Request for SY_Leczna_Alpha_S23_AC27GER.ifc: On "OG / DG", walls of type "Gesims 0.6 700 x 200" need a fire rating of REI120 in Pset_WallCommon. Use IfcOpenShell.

First a look at what the model holds.

```python
import ifcopenshell
import ifcopenshell.util.element

model = ifcopenshell.open("SY_Leczna_Alpha_S23_AC27GER.ifc")
print(model.schema)
storey = next(s for s in model.by_type("IfcBuildingStorey") if s.Name == "OG / DG")
walls = [e for e in ifcopenshell.util.element.get_decomposition(storey) if e.is_a("IfcWall")]
seen = {}
for e in walls:
    element_type = ifcopenshell.util.element.get_type(e)
    key = (element_type.Name if element_type != e and element_type else None, ifcopenshell.util.element.get_pset(e, "Pset_WallCommon", "FireRating"))
    seen[key] = seen.get(key, 0) + 1
for (name, value), count in sorted(seen.items(), key=str):
    print(count, "x", name, "|", value)
```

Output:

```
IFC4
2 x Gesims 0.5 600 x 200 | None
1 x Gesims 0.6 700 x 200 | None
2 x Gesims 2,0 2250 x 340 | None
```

```python
import ifcopenshell
import ifcopenshell.api.pset
import ifcopenshell.util.element

model = ifcopenshell.open("SY_Leczna_Alpha_S23_AC27GER.ifc")

storey = next(s for s in model.by_type("IfcBuildingStorey") if s.Name == "OG / DG")
walls = [e for e in ifcopenshell.util.element.get_decomposition(storey) if e.is_a("IfcWall")]

count = 0
for e in walls:
    element_type = ifcopenshell.util.element.get_type(e)
    if element_type in (None, e) or element_type.Name != "Gesims 0.6 700 x 200":
        continue
    # add_pset returns the element's existing set when there is one.
    pset = ifcopenshell.api.pset.add_pset(model, product=e, name="Pset_WallCommon")
    ifcopenshell.api.pset.edit_pset(model, pset=pset, properties={"FireRating": "REI120"})
    count += 1

print(count, "walls updated")

model.write("SY_Leczna_Alpha_S23_AC27GER_v2.ifc")
```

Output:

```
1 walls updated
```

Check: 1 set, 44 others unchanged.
